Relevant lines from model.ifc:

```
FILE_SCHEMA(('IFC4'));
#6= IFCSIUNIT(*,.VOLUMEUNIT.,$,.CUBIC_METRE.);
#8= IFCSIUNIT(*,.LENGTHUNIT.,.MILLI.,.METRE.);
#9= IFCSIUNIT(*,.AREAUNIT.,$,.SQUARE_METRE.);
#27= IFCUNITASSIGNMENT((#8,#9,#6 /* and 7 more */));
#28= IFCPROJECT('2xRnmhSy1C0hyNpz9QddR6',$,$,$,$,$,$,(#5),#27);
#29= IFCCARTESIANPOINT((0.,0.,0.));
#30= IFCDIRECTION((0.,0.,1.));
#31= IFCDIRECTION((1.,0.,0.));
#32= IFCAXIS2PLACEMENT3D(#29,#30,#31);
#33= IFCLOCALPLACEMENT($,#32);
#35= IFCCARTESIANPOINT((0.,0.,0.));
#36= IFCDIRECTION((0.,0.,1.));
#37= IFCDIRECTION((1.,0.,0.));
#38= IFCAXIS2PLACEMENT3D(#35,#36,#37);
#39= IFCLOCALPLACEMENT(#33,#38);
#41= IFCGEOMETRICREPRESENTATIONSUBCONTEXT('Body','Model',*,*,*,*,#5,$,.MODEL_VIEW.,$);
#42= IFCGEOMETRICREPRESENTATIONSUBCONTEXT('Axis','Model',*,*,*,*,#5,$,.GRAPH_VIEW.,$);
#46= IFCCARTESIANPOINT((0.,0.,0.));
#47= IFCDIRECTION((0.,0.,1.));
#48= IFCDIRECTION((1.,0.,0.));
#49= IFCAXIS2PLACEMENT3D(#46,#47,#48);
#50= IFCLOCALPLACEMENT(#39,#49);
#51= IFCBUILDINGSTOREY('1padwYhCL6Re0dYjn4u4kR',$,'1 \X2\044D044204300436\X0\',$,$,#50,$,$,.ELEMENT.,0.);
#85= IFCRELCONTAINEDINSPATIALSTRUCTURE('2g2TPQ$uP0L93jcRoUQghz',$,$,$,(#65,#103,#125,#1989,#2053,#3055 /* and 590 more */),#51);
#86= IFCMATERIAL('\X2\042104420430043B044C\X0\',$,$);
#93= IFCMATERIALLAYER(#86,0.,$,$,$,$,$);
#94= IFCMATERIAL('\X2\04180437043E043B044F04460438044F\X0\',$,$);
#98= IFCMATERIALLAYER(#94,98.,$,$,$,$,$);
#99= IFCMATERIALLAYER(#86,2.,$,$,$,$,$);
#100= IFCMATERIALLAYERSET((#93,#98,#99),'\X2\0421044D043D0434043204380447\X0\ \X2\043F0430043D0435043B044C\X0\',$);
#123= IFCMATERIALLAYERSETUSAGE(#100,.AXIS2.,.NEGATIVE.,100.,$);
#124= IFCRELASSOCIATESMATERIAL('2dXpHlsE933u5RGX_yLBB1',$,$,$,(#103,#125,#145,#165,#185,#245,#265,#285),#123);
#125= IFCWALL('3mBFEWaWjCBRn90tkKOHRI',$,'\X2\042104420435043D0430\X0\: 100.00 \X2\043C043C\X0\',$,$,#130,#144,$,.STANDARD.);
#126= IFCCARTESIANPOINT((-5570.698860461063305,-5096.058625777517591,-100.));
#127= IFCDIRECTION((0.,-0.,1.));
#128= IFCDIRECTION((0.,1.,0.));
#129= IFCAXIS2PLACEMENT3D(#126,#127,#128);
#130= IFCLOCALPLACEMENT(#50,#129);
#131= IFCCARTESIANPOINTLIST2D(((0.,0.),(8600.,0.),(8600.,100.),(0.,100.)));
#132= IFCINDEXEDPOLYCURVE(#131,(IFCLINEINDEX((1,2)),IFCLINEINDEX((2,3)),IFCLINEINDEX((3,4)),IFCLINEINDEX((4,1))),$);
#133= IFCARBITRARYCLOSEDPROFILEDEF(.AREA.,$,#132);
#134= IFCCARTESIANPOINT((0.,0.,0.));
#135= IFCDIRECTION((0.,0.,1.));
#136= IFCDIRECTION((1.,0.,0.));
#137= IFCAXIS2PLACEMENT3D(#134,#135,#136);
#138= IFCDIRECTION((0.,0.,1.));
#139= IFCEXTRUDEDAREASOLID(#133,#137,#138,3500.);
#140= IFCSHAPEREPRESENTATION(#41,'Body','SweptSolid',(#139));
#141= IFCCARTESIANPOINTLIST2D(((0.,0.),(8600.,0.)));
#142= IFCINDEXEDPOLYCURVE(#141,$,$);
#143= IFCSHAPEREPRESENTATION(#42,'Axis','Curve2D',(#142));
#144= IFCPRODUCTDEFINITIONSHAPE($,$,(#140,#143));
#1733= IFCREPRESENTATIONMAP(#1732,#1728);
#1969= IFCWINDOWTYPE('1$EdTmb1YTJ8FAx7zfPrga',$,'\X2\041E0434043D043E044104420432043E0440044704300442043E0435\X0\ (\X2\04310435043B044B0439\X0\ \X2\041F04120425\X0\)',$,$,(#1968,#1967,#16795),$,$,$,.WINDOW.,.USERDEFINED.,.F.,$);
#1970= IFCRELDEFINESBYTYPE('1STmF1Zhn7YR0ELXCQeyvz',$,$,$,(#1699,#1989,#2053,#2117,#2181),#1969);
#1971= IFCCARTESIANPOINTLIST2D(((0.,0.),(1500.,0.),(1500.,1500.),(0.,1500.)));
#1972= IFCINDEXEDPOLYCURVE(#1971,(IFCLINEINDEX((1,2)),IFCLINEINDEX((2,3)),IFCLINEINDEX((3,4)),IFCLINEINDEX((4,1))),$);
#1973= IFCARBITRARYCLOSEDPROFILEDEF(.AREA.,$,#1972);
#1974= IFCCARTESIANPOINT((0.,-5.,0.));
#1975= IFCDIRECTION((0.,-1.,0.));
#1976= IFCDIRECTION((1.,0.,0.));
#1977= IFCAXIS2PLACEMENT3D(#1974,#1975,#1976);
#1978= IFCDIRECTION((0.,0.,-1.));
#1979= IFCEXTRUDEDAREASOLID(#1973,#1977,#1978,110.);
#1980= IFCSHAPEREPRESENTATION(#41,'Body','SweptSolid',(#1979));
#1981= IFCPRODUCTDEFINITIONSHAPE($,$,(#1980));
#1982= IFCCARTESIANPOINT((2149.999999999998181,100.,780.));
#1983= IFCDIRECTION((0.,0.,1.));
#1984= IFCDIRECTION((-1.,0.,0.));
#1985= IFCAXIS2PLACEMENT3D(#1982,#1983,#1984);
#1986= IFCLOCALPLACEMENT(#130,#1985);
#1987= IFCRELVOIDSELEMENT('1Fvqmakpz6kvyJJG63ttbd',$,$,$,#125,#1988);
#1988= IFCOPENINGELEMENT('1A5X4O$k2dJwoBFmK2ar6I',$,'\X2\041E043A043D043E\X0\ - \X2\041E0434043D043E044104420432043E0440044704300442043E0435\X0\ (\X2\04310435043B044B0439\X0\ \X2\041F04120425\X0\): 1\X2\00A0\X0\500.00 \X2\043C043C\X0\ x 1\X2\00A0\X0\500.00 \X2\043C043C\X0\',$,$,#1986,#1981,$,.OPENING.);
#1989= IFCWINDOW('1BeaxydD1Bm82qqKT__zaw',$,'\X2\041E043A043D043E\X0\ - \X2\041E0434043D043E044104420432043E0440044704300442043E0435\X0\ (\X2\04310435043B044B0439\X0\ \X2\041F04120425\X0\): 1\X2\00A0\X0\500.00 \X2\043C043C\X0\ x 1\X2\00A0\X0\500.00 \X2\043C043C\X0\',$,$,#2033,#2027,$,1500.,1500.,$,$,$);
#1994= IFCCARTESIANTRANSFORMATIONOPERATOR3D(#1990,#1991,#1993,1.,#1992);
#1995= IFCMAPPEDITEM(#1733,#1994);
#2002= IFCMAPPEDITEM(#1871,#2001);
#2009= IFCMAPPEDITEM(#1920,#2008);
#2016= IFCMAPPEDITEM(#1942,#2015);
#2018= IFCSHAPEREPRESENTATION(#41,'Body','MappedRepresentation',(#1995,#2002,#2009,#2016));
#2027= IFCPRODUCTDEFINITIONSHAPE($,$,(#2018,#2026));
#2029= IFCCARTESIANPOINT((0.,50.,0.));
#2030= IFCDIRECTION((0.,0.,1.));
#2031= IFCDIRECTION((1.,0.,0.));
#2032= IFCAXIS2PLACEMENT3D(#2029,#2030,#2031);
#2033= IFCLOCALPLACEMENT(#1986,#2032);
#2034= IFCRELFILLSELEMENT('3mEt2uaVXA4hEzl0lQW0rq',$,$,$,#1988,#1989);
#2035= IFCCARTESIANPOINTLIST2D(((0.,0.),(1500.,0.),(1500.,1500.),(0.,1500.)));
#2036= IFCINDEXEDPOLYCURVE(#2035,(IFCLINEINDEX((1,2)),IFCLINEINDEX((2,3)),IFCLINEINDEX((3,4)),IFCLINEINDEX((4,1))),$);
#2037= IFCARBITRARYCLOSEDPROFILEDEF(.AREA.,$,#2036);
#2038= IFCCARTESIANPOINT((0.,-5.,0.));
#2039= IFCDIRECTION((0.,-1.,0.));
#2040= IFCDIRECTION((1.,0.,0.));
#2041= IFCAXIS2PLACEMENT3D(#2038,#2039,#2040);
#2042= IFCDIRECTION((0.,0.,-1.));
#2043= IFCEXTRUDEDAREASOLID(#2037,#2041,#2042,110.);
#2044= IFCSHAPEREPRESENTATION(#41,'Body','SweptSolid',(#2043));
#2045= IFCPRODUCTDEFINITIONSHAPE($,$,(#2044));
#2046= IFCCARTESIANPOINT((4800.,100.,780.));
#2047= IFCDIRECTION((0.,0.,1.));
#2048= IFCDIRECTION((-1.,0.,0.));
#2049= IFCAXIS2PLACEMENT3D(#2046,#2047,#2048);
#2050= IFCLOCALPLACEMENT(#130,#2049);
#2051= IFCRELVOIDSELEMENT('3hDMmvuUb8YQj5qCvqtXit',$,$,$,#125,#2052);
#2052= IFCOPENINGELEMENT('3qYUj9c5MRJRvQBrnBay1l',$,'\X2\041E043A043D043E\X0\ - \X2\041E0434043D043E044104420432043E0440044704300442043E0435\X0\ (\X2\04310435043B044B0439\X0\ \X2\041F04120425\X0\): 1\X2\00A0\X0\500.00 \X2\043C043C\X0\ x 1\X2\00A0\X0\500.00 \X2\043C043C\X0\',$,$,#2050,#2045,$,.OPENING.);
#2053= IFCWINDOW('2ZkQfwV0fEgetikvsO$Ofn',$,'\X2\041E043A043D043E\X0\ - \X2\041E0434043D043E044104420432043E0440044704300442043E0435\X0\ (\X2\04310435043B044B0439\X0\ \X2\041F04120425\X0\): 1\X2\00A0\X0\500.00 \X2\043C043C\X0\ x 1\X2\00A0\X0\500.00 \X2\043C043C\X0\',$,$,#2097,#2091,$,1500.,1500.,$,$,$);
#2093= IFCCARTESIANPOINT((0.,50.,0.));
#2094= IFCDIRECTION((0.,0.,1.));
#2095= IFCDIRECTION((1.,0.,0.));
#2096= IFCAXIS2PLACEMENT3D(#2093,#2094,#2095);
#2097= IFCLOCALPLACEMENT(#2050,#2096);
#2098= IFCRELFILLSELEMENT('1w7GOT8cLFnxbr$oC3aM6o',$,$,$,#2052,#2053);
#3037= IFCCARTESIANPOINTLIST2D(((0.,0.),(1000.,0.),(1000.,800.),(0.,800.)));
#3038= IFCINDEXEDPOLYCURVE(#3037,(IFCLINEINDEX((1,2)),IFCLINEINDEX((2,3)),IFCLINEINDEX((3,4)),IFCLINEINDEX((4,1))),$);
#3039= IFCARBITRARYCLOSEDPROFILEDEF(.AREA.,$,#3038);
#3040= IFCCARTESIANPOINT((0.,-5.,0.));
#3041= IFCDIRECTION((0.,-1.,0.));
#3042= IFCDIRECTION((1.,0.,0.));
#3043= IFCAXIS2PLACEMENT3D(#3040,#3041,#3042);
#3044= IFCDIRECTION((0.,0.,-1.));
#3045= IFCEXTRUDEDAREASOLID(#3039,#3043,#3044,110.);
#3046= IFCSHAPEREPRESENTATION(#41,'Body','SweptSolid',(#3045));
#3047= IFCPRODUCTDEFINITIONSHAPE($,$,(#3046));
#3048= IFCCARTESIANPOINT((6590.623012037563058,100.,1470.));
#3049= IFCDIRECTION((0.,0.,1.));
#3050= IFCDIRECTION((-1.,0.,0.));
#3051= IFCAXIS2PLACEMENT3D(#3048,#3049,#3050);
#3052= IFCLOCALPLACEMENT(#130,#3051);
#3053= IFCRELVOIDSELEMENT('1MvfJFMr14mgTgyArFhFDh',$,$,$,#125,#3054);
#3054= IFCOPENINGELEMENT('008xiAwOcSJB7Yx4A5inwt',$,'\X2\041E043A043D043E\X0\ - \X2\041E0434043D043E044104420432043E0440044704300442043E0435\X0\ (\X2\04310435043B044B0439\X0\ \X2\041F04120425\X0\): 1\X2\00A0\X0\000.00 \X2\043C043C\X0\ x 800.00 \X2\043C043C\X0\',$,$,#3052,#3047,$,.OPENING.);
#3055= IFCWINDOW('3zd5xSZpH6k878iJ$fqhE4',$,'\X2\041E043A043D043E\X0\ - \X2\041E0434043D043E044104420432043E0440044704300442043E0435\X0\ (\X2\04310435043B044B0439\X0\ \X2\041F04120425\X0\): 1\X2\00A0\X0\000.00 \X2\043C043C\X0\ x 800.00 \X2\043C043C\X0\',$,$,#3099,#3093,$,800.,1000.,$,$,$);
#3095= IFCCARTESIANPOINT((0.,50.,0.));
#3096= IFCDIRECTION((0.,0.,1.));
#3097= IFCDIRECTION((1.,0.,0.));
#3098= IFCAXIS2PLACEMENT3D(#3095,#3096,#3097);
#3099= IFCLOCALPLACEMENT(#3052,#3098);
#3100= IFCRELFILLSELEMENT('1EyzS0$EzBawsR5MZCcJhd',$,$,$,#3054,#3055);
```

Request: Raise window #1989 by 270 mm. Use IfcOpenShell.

```python
import numpy as np
import ifcopenshell
import ifcopenshell.api.geometry
import ifcopenshell.util.placement
import ifcopenshell.util.unit

model = ifcopenshell.open("model.ifc")
unit_scale = ifcopenshell.util.unit.calculate_unit_scale(model)

window = model.by_guid("1BeaxydD1Bm82qqKT__zaw")
opening = window.FillsVoids[0].RelatingOpeningElement
dz = 270.0

shift = np.array([0.0, 0.0, dz])
# The window is placed relative to its opening, so it follows when the opening moves.
matrix = ifcopenshell.util.placement.get_local_placement(opening.ObjectPlacement)
matrix[:3, 3] += shift
ifcopenshell.api.geometry.edit_object_placement(
    model, product=opening, matrix=matrix, is_si=False, should_transform_children=True
)

print(f"moved by {dz * unit_scale:+.3f} m")

model.write("model_v2.ifc")
```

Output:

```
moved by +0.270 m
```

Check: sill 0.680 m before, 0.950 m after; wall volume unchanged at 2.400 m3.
